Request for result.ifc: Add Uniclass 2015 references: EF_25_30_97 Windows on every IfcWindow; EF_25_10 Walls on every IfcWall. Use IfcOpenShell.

First a look at what the model holds.

```python
import ifcopenshell

model = ifcopenshell.open("result.ifc")
print(model.schema)
print("classifications:", [c.Name for c in model.by_type("IfcClassification")])
for ifc_class in ("IfcDoor", "IfcRoof", "IfcStair", "IfcWall", "IfcWindow"):
    print(ifc_class, len(model.by_type(ifc_class)))
```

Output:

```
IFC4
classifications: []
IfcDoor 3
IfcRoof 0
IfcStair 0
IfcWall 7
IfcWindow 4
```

```python
import ifcopenshell
import ifcopenshell.api.classification

model = ifcopenshell.open("result.ifc")

system = ifcopenshell.api.classification.add_classification(model, classification="Uniclass 2015")

codes = {
    "IfcWindow": ("EF_25_30_97", "Windows"),
    "IfcWall": ("EF_25_10", "Walls"),
}
for ifc_class, (code, name) in codes.items():
    products = model.by_type(ifc_class)
    ifcopenshell.api.classification.add_reference(
        model, products=products, classification=system, identification=code, name=name
    )
    print(code, len(products))

model.write("result_edited.ifc")
```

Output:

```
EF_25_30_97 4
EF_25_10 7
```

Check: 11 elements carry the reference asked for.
